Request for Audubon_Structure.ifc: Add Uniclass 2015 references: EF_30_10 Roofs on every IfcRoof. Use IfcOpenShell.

First a look at what the model holds.

```python
import ifcopenshell

model = ifcopenshell.open("Audubon_Structure.ifc")
print(model.schema)
print("classifications:", [c.Name for c in model.by_type("IfcClassification")])
for ifc_class in ("IfcDoor", "IfcRoof", "IfcStair", "IfcWall", "IfcWindow"):
    print(ifc_class, len(model.by_type(ifc_class)))
```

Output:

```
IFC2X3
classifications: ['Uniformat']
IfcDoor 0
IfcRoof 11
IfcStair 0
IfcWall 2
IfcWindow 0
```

```python
import ifcopenshell
import ifcopenshell.api.classification

model = ifcopenshell.open("Audubon_Structure.ifc")

# IFC2X3 requires Source and Edition and has no link from the project to the system.
system = model.create_entity("IfcClassification", Source="NBS", Edition="2015", Name="Uniclass 2015")

codes = {
    "IfcRoof": ("EF_30_10", "Roofs"),
}
for ifc_class, (code, name) in codes.items():
    products = model.by_type(ifc_class)
    ifcopenshell.api.classification.add_reference(
        model, products=products, classification=system, identification=code, name=name
    )
    print(code, len(products))

model.write("Audubon_Structure-out.ifc")
```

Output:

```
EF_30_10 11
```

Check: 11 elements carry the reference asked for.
